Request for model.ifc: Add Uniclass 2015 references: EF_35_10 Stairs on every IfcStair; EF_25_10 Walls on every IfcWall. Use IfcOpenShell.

First a look at what the model holds.

```python
import ifcopenshell

model = ifcopenshell.open("model.ifc")
print(model.schema)
print("classifications:", [c.Name for c in model.by_type("IfcClassification")])
for ifc_class in ("IfcDoor", "IfcRoof", "IfcStair", "IfcWall", "IfcWindow"):
    print(ifc_class, len(model.by_type(ifc_class)))
```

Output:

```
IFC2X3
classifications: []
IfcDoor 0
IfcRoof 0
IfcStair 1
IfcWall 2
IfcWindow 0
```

```python
import ifcopenshell
import ifcopenshell.api.classification

model = ifcopenshell.open("model.ifc")

# IFC2X3 requires Source and Edition and has no link from the project to the system.
system = model.create_entity("IfcClassification", Source="NBS", Edition="2015", Name="Uniclass 2015")

codes = {
    "IfcStair": ("EF_35_10", "Stairs"),
    "IfcWall": ("EF_25_10", "Walls"),
}
for ifc_class, (code, name) in codes.items():
    products = model.by_type(ifc_class)
    ifcopenshell.api.classification.add_reference(
        model, products=products, classification=system, identification=code, name=name
    )
    print(code, len(products))

model.write("model_rev.ifc")
```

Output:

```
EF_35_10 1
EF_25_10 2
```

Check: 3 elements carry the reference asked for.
